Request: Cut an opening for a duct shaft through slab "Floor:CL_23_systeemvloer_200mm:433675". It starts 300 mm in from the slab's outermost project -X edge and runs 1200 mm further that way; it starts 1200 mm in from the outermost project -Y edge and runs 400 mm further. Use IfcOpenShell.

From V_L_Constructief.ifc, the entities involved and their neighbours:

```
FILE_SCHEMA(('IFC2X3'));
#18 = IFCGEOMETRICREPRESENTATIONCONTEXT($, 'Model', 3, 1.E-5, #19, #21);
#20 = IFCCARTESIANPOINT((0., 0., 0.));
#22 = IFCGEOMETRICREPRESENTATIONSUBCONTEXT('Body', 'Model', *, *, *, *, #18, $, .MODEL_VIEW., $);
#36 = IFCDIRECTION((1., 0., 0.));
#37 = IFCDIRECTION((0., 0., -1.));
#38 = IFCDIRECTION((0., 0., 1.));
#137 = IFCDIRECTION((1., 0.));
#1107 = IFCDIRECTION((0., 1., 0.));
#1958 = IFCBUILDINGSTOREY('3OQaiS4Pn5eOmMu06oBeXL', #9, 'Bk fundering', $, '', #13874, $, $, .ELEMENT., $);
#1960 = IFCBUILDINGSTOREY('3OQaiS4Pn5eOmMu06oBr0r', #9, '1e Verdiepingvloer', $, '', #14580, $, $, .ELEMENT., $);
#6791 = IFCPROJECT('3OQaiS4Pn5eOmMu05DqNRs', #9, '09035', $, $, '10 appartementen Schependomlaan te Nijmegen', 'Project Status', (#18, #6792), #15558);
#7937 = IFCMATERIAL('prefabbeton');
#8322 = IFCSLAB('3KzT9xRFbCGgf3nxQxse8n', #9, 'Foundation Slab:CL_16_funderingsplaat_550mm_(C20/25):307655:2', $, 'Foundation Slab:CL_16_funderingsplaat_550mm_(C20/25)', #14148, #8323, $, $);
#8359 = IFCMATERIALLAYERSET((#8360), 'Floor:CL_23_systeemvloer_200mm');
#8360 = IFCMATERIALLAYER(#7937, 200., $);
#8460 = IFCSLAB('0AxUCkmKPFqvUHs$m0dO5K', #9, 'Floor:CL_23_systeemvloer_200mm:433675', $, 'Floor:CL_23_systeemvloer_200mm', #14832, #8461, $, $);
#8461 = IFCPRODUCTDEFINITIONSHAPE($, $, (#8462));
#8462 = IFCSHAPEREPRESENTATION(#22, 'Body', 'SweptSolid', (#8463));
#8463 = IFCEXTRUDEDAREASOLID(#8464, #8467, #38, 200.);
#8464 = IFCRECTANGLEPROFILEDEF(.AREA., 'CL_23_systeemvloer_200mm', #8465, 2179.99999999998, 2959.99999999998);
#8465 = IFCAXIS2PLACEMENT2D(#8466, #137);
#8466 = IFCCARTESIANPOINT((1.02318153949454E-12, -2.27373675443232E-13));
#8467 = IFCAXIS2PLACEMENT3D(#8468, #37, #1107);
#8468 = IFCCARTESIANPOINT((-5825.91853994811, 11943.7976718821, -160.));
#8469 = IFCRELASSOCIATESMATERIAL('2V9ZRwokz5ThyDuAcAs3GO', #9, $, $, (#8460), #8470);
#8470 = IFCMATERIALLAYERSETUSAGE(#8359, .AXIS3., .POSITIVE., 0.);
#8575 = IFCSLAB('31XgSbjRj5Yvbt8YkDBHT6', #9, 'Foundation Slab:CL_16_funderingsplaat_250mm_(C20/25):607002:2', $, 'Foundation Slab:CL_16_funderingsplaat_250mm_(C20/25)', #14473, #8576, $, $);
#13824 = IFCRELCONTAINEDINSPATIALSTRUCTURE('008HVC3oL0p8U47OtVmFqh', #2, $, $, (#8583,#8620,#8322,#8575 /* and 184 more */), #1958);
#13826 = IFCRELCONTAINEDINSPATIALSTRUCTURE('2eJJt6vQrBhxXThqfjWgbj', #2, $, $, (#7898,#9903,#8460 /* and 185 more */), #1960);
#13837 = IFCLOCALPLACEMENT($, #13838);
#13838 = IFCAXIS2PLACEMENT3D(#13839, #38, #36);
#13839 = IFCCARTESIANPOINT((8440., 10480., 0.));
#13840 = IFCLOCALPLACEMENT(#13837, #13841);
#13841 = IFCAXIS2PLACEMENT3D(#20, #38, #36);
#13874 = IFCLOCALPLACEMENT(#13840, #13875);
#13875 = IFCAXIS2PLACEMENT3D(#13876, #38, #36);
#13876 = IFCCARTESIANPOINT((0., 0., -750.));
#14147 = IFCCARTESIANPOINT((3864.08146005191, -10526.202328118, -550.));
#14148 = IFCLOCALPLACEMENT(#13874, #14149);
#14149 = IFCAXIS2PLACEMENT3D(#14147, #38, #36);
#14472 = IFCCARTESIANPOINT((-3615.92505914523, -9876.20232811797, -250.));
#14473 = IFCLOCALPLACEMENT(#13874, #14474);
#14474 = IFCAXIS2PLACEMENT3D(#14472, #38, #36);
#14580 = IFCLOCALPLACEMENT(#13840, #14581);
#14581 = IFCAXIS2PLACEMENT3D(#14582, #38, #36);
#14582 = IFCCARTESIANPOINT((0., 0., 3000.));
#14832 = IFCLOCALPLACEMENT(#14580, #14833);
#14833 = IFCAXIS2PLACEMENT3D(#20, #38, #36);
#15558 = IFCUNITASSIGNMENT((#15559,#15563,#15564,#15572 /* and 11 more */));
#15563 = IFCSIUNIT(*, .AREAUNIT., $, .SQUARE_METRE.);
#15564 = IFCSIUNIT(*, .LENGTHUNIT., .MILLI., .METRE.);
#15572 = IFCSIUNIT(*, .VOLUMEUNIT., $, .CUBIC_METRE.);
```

```python
import numpy as np
import ifcopenshell
import ifcopenshell.api.feature
import ifcopenshell.api.geometry
import ifcopenshell.api.root
import ifcopenshell.geom
import ifcopenshell.util.placement
import ifcopenshell.util.representation
import ifcopenshell.util.shape
import ifcopenshell.util.unit

model = ifcopenshell.open("V_L_Constructief.ifc")
unit_scale = ifcopenshell.util.unit.calculate_unit_scale(model)
settings = ifcopenshell.geom.settings()


def volume(element):
    """Net volume in cubic metres, openings subtracted."""
    shape = ifcopenshell.geom.create_shape(settings, element)
    return ifcopenshell.util.shape.get_volume(shape.geometry)


slab = model.by_id(8460)
before = volume(slab)

# Extent in the slab's own axes, in metres. The edges named are its -X and -Y sides.
slab_shape = ifcopenshell.geom.create_shape(settings, slab)
vertices = ifcopenshell.util.shape.get_vertices(slab_shape.geometry)
x_min, y_min, bottom = vertices.min(axis=0)
top = vertices[:, 2].max()

opening = ifcopenshell.api.root.create_entity(model, ifc_class="IfcOpeningElement", name="Duct shaft opening")
context = ifcopenshell.util.representation.get_context(model, "Model", "Body", "MODEL_VIEW")
width, depth = 1.2, 0.4
outline = [(0.0, 0.0), (width, 0.0), (width, depth), (0.0, depth), (0.0, 0.0)]
# Overshoot both faces by 50 mm so the cut is clean.
shape = ifcopenshell.api.geometry.add_slab_representation(
    model, context=context, depth=top - bottom + 0.1, polyline=outline
)
ifcopenshell.api.geometry.assign_representation(model, product=opening, representation=shape)

matrix = ifcopenshell.util.placement.get_local_placement(slab.ObjectPlacement)
matrix[:, 3] = matrix @ np.append(np.array([x_min + 0.3, y_min + 1.2, bottom - 0.05]) / unit_scale, 1.0)
ifcopenshell.api.geometry.edit_object_placement(model, product=opening, matrix=matrix, is_si=False)
ifcopenshell.api.feature.add_feature(model, feature=opening, element=slab)

after = volume(slab)

print(f"slab volume {before:.3f} -> {after:.3f} m3")

model.write("V_L_Constructief_rev.ifc")
```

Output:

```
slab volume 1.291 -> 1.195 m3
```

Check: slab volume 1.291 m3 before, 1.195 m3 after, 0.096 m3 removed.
